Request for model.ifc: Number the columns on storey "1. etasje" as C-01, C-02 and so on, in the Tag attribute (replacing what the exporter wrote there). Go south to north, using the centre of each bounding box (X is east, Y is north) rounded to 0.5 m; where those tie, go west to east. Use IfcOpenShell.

First a look at what the model holds.

```python
import ifcopenshell
import ifcopenshell.util.element
import ifcopenshell.util.placement

model = ifcopenshell.open("model.ifc")
print(model.schema)
storey = next(s for s in model.by_type("IfcBuildingStorey") if s.Name == "1. etasje")
columns = [e for e in ifcopenshell.util.element.get_decomposition(storey) if e.is_a("IfcColumn")]
for e in sorted(columns, key=lambda e: e.id()):
    origin = ifcopenshell.util.placement.get_local_placement(e.ObjectPlacement)[:3, 3]
    print(e.id(), e.Tag, e.Name, origin.round(2) + 0.0, sep=" | ")
```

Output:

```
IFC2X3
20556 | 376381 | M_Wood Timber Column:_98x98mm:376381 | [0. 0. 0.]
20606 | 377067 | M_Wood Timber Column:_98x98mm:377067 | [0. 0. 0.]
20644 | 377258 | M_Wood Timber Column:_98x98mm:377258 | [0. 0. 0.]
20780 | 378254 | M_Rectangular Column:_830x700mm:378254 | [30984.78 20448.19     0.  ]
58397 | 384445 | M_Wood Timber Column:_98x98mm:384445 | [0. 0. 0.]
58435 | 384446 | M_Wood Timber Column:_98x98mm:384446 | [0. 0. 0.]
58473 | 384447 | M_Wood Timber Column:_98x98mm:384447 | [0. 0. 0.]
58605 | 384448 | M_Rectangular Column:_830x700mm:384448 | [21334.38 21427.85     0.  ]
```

```python
import ifcopenshell
import ifcopenshell.geom
import ifcopenshell.util.element
import ifcopenshell.util.shape

model = ifcopenshell.open("model.ifc")
settings = ifcopenshell.geom.settings()
settings.set("use-world-coords", True)


def centre(element):
    shape = ifcopenshell.geom.create_shape(settings, element)
    return ifcopenshell.util.shape.get_bbox_centroid(shape.geometry)


storey = next(s for s in model.by_type("IfcBuildingStorey") if s.Name == "1. etasje")
columns = [e for e in ifcopenshell.util.element.get_decomposition(storey) if e.is_a("IfcColumn")]

# Insertion points can sit at a corner or the storey origin, so sort by the geometry (in metres).
centres = {e: centre(e) for e in columns}
columns.sort(key=lambda e: (round(centres[e][1] / 0.5), centres[e][0]))

for i, e in enumerate(columns, start=1):
    number = f"C-{i:02d}"
    e.Tag = number
    print(e.id(), number)

model.write("model_v2.ifc")
```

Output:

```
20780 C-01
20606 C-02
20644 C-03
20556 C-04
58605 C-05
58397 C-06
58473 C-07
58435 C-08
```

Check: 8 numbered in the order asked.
